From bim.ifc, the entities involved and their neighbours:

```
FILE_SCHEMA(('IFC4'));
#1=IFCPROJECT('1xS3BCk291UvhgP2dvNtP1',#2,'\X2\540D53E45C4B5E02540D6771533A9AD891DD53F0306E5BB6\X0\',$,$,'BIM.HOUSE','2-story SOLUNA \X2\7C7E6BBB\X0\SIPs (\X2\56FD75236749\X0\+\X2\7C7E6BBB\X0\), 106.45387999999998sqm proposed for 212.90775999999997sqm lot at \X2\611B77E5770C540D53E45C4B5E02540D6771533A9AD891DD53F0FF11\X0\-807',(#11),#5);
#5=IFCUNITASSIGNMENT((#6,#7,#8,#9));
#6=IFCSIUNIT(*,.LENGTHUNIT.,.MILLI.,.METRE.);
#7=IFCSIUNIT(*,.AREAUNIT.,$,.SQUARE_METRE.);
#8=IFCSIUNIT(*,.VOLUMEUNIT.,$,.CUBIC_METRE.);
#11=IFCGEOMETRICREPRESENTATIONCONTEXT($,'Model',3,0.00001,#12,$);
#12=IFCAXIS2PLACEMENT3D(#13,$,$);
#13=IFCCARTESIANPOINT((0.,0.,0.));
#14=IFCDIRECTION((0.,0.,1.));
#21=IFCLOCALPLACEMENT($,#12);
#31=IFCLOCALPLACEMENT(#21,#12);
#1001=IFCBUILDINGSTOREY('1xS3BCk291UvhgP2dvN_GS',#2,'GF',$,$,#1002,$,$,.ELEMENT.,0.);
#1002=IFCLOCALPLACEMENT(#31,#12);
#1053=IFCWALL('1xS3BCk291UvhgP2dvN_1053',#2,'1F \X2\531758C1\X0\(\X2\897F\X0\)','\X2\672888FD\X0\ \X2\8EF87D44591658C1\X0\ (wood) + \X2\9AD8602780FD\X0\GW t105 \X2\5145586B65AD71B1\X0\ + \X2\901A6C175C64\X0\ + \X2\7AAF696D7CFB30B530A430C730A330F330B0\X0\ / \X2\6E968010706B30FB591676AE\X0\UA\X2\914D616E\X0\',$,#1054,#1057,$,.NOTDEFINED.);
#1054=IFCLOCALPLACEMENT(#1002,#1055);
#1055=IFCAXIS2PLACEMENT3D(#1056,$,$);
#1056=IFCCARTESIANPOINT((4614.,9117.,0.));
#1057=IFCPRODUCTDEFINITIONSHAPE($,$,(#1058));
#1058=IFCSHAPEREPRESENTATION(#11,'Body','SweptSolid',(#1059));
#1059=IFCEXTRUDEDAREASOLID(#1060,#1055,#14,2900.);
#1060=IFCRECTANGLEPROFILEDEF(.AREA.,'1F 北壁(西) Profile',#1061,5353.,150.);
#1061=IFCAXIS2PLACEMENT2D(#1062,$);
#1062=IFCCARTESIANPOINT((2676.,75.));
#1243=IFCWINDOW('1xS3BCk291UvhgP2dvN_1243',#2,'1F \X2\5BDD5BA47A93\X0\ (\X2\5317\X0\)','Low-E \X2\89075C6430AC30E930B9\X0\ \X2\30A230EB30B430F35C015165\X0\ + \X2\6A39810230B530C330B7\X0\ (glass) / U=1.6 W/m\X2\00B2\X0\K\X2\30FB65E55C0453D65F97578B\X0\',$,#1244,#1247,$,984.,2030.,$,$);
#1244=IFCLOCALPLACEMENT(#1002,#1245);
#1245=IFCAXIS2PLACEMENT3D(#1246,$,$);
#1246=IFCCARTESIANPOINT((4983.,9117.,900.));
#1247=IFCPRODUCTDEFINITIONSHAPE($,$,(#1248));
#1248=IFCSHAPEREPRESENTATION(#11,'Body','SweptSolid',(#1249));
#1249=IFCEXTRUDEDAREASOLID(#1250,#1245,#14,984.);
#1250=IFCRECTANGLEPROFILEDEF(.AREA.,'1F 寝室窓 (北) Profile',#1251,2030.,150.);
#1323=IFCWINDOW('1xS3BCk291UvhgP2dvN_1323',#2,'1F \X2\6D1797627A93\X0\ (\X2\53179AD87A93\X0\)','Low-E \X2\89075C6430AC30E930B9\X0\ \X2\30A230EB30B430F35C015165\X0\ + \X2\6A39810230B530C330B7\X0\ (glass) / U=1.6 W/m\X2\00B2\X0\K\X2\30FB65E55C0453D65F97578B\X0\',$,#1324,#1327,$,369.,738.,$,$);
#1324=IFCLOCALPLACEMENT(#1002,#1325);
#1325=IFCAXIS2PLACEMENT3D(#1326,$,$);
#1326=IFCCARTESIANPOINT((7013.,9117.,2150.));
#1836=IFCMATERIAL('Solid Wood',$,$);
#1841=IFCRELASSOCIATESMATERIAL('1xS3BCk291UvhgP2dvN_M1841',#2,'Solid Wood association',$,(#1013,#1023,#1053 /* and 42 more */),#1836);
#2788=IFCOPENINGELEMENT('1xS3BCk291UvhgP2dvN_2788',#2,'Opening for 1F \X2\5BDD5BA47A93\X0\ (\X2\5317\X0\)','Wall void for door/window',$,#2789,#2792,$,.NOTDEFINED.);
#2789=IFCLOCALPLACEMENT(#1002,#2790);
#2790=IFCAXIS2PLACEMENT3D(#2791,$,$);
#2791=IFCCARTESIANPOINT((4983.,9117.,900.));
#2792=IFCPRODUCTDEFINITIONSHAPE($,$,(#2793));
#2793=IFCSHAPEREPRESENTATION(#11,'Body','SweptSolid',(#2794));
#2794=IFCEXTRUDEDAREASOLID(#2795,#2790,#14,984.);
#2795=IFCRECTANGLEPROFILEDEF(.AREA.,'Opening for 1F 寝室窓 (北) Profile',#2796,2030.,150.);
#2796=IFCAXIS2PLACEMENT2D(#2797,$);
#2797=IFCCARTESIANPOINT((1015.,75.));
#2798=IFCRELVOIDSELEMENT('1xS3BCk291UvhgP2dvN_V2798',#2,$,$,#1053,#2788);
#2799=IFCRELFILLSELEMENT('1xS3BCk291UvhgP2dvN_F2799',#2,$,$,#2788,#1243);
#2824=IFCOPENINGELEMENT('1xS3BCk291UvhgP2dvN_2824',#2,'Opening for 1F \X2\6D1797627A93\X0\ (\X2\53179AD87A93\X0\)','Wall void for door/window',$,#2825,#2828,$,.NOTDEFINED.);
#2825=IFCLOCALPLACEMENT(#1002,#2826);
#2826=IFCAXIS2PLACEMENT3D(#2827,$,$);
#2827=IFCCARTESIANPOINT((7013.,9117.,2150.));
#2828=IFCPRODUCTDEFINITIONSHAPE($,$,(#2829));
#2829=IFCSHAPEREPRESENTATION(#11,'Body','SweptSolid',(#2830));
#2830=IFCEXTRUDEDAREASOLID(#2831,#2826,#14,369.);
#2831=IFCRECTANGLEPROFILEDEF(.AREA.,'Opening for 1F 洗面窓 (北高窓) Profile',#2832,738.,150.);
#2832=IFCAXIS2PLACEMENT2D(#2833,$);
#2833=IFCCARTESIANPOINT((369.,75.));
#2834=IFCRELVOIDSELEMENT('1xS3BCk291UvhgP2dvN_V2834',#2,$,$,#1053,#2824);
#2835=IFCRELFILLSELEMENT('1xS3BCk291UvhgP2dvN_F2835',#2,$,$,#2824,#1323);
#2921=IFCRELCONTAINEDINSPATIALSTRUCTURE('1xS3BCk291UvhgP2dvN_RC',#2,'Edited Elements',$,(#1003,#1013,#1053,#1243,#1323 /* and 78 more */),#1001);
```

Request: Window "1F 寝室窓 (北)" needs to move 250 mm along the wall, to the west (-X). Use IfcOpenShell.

```python
import ifcopenshell
import ifcopenshell.api.geometry
import ifcopenshell.util.placement
import ifcopenshell.util.unit

model = ifcopenshell.open("bim.ifc")
unit_scale = ifcopenshell.util.unit.calculate_unit_scale(model)

window = model.by_guid("1xS3BCk291UvhgP2dvN_1243")
opening = window.FillsVoids[0].RelatingOpeningElement
wall = opening.VoidsElements[0].RelatingBuildingElement

wall_matrix = ifcopenshell.util.placement.get_local_placement(wall.ObjectPlacement)
shift = wall_matrix[:3, 0] * -0.25 / unit_scale
before = ifcopenshell.util.placement.get_local_placement(window.ObjectPlacement)[:3, 3].copy()

# The window is not placed relative to its opening, so move both.
for product in (opening, window):
    matrix = ifcopenshell.util.placement.get_local_placement(product.ObjectPlacement)
    matrix[:3, 3] += shift
    ifcopenshell.api.geometry.edit_object_placement(model, product=product, matrix=matrix, is_si=False)

after = ifcopenshell.util.placement.get_local_placement(window.ObjectPlacement)[:3, 3]
print("window moved by", (after - before).round(3) + 0.0)

model.write("bim-out.ifc")
```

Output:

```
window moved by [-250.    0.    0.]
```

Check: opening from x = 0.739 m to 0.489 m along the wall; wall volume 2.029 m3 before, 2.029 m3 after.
